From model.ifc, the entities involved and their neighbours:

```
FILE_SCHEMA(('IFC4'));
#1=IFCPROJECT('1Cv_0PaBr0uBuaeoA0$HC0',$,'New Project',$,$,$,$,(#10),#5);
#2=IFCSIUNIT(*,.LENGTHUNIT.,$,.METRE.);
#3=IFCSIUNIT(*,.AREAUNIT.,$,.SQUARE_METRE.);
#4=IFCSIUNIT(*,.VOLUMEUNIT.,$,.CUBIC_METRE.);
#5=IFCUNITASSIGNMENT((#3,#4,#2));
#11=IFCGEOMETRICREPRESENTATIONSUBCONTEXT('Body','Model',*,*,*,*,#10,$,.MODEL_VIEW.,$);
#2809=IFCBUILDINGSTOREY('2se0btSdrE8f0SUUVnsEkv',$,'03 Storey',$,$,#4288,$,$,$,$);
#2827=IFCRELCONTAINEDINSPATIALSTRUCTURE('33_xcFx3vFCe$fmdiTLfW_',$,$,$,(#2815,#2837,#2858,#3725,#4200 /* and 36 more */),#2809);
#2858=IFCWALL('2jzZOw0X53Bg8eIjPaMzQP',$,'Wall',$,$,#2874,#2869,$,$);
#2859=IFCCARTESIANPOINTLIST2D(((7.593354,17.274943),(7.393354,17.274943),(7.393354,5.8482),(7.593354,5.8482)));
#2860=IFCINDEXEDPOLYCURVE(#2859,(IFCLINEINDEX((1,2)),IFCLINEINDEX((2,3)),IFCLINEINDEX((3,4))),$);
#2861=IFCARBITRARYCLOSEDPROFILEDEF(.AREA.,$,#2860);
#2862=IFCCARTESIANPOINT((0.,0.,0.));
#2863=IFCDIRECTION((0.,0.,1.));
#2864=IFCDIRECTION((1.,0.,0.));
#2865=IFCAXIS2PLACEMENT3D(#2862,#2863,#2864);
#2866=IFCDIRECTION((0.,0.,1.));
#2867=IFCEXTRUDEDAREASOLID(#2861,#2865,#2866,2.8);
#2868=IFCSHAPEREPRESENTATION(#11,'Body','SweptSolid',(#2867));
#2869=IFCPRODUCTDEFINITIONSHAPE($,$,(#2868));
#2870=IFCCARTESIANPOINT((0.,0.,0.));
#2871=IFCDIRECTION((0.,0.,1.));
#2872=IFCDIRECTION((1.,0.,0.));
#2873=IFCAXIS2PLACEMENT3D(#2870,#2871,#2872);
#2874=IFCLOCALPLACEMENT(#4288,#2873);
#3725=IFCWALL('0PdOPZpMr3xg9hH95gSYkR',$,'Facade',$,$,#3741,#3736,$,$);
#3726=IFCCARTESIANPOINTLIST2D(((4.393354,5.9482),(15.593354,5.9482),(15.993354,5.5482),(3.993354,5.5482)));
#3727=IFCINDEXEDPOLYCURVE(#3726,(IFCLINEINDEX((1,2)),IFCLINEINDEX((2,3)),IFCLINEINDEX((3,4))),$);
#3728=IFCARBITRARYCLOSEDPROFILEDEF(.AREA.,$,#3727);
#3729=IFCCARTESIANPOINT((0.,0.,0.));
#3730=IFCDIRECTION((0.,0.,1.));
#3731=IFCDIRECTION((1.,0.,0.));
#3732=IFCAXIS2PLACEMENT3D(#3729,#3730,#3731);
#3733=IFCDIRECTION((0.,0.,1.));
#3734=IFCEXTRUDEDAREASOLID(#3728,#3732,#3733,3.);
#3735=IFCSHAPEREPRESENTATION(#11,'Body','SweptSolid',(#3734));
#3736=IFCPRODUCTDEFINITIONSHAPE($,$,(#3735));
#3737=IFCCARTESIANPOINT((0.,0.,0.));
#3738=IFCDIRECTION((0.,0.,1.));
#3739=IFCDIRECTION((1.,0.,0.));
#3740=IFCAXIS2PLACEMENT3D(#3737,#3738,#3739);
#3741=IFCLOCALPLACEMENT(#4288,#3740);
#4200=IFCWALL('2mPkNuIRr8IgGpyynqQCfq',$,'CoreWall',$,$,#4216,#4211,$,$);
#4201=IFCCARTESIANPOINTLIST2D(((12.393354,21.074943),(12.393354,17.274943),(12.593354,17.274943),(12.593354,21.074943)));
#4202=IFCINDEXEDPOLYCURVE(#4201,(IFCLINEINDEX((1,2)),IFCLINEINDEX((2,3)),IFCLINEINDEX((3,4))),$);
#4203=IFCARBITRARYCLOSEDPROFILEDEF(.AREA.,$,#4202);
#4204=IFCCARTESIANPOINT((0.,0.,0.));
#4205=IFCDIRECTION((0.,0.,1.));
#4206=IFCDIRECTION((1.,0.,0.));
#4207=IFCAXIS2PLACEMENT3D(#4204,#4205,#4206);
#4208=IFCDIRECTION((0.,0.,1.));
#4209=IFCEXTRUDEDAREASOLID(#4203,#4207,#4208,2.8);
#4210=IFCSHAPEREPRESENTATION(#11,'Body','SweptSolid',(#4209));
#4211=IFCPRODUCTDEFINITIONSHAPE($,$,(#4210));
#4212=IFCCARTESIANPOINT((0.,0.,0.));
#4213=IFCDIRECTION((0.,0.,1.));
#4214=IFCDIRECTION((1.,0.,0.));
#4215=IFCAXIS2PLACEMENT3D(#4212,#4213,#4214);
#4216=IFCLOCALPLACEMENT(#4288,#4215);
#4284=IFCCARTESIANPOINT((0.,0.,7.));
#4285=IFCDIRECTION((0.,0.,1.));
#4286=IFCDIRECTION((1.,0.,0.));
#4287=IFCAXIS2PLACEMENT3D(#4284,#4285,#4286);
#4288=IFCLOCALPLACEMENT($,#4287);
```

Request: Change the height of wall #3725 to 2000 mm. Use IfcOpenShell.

```python
import ifcopenshell
import ifcopenshell.geom
import ifcopenshell.util.representation
import ifcopenshell.util.shape

model = ifcopenshell.open("model.ifc")
settings = ifcopenshell.geom.settings()


def volume(element):
    """Net volume in cubic metres, openings subtracted."""
    shape = ifcopenshell.geom.create_shape(settings, element)
    return ifcopenshell.util.shape.get_volume(shape.geometry)


wall = model.by_guid("0PdOPZpMr3xg9hH95gSYkR")
before = volume(wall)

body = ifcopenshell.util.representation.get_representation(wall, "Model", "Body")
solid = body.Items[0]
old_height = solid.Depth
solid.Depth = 2.0
after = volume(wall)

print(f"height {old_height:g} -> {solid.Depth:g}, volume {before:.3f} -> {after:.3f} m3")

model.write("model_edited.ifc")
```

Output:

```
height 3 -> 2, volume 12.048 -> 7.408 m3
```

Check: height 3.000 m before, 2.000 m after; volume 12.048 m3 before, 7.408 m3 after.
